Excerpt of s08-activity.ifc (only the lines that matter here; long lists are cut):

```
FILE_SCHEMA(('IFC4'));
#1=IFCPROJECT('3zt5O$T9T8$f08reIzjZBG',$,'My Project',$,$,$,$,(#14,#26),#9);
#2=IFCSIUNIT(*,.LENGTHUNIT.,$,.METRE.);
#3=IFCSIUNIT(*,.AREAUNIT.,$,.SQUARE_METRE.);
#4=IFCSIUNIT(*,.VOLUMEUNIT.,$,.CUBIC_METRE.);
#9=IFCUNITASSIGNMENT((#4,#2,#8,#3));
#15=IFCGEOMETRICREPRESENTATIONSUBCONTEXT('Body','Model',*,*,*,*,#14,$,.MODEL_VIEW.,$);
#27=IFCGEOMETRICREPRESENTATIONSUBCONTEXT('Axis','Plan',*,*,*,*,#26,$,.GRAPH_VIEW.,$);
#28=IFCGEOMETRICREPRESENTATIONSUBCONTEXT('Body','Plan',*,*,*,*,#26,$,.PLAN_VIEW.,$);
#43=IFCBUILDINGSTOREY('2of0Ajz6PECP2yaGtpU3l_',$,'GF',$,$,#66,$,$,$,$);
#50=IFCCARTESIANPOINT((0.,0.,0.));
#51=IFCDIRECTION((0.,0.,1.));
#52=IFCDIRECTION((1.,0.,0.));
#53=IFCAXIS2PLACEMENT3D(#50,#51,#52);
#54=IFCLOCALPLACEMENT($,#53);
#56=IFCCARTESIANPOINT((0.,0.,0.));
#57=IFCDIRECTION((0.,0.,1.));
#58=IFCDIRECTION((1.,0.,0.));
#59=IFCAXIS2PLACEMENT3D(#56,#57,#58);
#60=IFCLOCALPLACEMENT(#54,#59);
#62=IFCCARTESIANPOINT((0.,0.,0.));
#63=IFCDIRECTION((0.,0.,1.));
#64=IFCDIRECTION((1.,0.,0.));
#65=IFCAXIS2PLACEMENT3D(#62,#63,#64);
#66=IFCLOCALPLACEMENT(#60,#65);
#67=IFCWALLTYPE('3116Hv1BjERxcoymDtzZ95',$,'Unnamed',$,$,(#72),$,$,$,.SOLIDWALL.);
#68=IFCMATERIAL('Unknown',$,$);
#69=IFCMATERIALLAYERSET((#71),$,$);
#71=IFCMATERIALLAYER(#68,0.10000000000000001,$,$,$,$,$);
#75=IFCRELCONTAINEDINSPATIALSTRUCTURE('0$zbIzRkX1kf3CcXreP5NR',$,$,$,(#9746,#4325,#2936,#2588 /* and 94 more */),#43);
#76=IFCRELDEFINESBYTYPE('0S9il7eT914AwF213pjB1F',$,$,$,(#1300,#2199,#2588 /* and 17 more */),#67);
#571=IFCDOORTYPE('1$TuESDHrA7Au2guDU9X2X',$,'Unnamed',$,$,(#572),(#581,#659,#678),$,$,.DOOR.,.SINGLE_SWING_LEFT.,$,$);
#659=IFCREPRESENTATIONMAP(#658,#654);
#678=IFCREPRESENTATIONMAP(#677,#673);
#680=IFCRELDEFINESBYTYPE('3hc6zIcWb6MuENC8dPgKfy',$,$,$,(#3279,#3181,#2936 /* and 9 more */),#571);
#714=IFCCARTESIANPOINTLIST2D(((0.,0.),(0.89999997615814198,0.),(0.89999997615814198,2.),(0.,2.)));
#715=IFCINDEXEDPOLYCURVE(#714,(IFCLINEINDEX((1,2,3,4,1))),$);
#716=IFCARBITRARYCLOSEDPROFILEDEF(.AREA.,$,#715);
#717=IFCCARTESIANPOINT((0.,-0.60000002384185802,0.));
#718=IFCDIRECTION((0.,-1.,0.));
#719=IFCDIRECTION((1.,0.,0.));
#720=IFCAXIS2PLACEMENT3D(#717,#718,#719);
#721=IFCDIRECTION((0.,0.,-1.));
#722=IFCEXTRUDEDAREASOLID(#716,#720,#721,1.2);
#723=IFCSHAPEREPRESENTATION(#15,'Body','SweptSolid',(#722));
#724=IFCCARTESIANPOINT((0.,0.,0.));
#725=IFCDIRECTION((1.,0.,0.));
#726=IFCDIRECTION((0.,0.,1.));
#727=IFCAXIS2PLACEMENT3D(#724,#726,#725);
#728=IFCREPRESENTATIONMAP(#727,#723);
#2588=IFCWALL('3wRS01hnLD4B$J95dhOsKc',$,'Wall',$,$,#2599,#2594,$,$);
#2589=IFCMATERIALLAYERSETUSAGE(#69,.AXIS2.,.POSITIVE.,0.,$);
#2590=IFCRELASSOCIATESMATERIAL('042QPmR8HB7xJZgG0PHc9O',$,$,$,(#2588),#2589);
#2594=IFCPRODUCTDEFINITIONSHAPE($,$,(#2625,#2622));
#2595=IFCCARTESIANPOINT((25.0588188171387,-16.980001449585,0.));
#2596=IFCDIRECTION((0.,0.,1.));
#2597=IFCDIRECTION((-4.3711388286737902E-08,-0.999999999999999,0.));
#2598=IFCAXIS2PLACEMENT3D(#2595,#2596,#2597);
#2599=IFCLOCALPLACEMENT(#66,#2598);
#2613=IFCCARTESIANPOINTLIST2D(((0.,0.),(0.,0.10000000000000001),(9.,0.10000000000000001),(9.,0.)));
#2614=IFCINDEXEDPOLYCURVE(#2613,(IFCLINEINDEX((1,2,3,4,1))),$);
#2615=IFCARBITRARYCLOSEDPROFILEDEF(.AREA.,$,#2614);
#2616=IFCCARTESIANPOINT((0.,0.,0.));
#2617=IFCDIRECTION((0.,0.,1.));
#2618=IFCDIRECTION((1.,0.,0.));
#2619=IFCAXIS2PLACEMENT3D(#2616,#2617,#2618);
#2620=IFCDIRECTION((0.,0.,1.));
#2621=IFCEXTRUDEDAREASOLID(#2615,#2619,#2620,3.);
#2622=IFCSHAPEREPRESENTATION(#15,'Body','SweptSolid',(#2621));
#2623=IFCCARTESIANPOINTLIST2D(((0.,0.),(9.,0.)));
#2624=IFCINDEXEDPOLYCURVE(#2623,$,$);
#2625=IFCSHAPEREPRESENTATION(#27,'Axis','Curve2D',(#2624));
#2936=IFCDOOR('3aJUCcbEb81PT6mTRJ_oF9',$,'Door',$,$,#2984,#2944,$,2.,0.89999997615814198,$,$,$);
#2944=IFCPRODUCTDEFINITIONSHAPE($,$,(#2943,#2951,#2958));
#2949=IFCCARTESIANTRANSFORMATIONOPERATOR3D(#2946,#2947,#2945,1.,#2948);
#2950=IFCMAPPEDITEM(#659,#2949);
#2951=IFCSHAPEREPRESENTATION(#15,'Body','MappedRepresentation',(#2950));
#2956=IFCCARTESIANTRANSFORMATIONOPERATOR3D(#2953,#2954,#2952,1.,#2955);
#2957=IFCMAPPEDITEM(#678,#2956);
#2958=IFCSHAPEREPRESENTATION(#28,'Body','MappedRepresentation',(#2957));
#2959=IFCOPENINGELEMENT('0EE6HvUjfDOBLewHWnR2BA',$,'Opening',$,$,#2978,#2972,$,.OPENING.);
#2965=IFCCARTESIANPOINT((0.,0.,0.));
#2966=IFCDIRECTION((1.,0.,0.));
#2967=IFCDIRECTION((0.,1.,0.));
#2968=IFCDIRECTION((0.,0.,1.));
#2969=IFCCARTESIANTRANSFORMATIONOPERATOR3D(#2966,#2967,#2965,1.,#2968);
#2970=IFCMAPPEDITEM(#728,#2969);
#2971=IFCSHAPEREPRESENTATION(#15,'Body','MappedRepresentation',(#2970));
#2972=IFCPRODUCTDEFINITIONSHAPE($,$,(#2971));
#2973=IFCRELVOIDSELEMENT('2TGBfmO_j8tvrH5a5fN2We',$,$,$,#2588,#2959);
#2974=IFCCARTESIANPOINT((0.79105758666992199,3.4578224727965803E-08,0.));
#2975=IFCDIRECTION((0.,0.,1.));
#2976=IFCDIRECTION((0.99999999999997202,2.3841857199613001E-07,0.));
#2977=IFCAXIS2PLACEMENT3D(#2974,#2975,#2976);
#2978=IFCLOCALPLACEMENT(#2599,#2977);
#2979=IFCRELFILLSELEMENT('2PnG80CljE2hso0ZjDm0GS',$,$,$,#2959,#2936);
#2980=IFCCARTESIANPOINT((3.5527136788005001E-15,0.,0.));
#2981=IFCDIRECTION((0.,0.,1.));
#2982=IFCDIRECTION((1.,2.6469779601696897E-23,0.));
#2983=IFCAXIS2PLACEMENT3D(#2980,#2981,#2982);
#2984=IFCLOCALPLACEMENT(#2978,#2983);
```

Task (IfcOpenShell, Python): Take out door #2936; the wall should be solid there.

```python
import ifcopenshell
import ifcopenshell.api.feature
import ifcopenshell.api.root
import ifcopenshell.geom
import ifcopenshell.util.shape

model = ifcopenshell.open("s08-activity.ifc")
settings = ifcopenshell.geom.settings()


def volume(element):
    """Net volume in cubic metres, openings subtracted."""
    shape = ifcopenshell.geom.create_shape(settings, element)
    return ifcopenshell.util.shape.get_volume(shape.geometry)


door = model.by_id(2936)
opening = door.FillsVoids[0].RelatingOpeningElement
wall = opening.VoidsElements[0].RelatingBuildingElement
before = volume(wall)

ifcopenshell.api.root.remove_product(model, product=door)
ifcopenshell.api.feature.remove_feature(model, feature=opening)

after = volume(wall)

print(f"wall volume {before:.3f} -> {after:.3f} m3")

model.write("s08-activity-out.ifc")
```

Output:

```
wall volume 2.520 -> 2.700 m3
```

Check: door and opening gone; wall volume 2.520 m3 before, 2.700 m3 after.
